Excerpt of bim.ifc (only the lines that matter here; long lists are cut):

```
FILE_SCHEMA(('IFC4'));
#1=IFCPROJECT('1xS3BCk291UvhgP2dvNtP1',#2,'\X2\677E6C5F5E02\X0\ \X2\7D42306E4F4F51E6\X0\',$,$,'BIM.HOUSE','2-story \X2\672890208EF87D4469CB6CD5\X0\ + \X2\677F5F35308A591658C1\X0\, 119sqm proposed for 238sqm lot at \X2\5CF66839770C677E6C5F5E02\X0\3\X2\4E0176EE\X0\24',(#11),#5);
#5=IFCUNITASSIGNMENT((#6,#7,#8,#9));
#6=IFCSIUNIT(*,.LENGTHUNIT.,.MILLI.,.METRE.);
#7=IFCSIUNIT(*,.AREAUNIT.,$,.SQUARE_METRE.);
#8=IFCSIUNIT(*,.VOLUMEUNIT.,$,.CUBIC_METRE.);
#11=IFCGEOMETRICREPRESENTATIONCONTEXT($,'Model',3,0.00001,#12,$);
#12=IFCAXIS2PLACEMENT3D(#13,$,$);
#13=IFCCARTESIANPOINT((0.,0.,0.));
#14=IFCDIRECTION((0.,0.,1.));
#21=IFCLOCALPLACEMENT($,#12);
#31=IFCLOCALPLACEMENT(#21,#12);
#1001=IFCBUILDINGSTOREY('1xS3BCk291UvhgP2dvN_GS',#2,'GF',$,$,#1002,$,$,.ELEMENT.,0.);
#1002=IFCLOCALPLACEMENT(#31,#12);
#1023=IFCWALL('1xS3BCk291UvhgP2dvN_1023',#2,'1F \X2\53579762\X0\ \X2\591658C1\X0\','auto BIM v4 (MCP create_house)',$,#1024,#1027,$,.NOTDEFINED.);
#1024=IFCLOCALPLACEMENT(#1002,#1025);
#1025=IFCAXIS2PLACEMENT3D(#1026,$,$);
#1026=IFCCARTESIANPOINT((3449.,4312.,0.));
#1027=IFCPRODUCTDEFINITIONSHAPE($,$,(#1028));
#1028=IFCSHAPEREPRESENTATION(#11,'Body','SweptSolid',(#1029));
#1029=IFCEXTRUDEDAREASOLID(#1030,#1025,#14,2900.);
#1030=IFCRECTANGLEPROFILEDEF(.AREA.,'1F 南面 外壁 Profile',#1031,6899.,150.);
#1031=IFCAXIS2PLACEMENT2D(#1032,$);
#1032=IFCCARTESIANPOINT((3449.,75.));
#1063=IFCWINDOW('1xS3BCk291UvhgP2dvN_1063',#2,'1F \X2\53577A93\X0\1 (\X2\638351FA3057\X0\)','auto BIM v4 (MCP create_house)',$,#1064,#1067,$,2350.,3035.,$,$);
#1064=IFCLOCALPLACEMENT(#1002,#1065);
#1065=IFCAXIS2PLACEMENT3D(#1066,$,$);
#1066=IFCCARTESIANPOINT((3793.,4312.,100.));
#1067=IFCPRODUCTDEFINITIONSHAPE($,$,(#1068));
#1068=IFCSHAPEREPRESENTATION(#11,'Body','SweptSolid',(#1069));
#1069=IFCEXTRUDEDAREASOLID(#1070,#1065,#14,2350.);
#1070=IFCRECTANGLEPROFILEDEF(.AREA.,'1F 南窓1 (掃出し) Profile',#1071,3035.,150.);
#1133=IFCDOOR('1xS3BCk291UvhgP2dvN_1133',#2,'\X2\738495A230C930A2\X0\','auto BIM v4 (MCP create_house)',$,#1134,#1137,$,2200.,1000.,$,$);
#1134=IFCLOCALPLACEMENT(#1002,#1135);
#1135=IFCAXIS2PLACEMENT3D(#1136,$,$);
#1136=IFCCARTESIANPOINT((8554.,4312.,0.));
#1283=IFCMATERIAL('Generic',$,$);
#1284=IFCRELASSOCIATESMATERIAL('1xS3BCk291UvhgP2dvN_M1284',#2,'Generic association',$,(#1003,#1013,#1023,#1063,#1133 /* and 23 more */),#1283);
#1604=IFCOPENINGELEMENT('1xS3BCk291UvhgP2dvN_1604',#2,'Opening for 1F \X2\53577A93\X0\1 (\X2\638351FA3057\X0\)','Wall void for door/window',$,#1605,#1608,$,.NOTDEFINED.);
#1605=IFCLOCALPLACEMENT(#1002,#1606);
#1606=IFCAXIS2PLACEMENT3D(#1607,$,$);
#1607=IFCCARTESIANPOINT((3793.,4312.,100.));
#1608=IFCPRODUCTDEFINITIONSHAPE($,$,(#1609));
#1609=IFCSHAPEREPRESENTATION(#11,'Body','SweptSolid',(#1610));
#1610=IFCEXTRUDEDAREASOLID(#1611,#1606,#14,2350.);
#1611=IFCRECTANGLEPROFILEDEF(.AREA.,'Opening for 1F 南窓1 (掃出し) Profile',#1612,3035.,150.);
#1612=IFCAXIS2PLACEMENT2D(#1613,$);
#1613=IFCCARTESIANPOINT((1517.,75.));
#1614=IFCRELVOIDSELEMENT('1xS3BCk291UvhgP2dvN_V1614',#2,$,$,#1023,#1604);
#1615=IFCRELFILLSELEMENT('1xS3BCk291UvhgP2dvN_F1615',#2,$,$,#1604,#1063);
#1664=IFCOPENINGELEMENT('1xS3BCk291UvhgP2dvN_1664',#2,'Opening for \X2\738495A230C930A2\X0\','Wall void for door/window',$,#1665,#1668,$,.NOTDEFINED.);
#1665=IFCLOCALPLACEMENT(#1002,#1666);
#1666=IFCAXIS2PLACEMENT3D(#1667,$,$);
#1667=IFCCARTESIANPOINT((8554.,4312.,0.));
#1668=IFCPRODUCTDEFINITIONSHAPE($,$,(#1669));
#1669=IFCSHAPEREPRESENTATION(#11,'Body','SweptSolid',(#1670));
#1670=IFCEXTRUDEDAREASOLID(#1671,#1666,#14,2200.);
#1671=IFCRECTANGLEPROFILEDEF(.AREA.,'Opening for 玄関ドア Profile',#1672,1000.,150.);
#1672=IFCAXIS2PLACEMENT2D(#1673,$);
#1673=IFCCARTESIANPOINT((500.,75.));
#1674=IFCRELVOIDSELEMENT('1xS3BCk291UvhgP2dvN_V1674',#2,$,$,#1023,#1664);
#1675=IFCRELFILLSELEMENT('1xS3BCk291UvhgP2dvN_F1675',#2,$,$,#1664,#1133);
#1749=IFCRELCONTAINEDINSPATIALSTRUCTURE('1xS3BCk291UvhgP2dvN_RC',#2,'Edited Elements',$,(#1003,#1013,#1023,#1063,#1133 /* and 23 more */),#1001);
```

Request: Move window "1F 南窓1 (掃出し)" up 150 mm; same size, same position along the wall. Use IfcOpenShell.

```python
import numpy as np
import ifcopenshell
import ifcopenshell.api.geometry
import ifcopenshell.util.placement
import ifcopenshell.util.unit

model = ifcopenshell.open("bim.ifc")
unit_scale = ifcopenshell.util.unit.calculate_unit_scale(model)

window = model.by_id(1063)
opening = window.FillsVoids[0].RelatingOpeningElement
dz = 0.15 / unit_scale

shift = np.array([0.0, 0.0, dz])
# The window is not placed relative to its opening, so move both.
for product in (opening, window):
    matrix = ifcopenshell.util.placement.get_local_placement(product.ObjectPlacement)
    matrix[:3, 3] += shift
    ifcopenshell.api.geometry.edit_object_placement(model, product=product, matrix=matrix, is_si=False)

print(f"moved by {dz * unit_scale:+.3f} m")

model.write("bim_edited.ifc")
```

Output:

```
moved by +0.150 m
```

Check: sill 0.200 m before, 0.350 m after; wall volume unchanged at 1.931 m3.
